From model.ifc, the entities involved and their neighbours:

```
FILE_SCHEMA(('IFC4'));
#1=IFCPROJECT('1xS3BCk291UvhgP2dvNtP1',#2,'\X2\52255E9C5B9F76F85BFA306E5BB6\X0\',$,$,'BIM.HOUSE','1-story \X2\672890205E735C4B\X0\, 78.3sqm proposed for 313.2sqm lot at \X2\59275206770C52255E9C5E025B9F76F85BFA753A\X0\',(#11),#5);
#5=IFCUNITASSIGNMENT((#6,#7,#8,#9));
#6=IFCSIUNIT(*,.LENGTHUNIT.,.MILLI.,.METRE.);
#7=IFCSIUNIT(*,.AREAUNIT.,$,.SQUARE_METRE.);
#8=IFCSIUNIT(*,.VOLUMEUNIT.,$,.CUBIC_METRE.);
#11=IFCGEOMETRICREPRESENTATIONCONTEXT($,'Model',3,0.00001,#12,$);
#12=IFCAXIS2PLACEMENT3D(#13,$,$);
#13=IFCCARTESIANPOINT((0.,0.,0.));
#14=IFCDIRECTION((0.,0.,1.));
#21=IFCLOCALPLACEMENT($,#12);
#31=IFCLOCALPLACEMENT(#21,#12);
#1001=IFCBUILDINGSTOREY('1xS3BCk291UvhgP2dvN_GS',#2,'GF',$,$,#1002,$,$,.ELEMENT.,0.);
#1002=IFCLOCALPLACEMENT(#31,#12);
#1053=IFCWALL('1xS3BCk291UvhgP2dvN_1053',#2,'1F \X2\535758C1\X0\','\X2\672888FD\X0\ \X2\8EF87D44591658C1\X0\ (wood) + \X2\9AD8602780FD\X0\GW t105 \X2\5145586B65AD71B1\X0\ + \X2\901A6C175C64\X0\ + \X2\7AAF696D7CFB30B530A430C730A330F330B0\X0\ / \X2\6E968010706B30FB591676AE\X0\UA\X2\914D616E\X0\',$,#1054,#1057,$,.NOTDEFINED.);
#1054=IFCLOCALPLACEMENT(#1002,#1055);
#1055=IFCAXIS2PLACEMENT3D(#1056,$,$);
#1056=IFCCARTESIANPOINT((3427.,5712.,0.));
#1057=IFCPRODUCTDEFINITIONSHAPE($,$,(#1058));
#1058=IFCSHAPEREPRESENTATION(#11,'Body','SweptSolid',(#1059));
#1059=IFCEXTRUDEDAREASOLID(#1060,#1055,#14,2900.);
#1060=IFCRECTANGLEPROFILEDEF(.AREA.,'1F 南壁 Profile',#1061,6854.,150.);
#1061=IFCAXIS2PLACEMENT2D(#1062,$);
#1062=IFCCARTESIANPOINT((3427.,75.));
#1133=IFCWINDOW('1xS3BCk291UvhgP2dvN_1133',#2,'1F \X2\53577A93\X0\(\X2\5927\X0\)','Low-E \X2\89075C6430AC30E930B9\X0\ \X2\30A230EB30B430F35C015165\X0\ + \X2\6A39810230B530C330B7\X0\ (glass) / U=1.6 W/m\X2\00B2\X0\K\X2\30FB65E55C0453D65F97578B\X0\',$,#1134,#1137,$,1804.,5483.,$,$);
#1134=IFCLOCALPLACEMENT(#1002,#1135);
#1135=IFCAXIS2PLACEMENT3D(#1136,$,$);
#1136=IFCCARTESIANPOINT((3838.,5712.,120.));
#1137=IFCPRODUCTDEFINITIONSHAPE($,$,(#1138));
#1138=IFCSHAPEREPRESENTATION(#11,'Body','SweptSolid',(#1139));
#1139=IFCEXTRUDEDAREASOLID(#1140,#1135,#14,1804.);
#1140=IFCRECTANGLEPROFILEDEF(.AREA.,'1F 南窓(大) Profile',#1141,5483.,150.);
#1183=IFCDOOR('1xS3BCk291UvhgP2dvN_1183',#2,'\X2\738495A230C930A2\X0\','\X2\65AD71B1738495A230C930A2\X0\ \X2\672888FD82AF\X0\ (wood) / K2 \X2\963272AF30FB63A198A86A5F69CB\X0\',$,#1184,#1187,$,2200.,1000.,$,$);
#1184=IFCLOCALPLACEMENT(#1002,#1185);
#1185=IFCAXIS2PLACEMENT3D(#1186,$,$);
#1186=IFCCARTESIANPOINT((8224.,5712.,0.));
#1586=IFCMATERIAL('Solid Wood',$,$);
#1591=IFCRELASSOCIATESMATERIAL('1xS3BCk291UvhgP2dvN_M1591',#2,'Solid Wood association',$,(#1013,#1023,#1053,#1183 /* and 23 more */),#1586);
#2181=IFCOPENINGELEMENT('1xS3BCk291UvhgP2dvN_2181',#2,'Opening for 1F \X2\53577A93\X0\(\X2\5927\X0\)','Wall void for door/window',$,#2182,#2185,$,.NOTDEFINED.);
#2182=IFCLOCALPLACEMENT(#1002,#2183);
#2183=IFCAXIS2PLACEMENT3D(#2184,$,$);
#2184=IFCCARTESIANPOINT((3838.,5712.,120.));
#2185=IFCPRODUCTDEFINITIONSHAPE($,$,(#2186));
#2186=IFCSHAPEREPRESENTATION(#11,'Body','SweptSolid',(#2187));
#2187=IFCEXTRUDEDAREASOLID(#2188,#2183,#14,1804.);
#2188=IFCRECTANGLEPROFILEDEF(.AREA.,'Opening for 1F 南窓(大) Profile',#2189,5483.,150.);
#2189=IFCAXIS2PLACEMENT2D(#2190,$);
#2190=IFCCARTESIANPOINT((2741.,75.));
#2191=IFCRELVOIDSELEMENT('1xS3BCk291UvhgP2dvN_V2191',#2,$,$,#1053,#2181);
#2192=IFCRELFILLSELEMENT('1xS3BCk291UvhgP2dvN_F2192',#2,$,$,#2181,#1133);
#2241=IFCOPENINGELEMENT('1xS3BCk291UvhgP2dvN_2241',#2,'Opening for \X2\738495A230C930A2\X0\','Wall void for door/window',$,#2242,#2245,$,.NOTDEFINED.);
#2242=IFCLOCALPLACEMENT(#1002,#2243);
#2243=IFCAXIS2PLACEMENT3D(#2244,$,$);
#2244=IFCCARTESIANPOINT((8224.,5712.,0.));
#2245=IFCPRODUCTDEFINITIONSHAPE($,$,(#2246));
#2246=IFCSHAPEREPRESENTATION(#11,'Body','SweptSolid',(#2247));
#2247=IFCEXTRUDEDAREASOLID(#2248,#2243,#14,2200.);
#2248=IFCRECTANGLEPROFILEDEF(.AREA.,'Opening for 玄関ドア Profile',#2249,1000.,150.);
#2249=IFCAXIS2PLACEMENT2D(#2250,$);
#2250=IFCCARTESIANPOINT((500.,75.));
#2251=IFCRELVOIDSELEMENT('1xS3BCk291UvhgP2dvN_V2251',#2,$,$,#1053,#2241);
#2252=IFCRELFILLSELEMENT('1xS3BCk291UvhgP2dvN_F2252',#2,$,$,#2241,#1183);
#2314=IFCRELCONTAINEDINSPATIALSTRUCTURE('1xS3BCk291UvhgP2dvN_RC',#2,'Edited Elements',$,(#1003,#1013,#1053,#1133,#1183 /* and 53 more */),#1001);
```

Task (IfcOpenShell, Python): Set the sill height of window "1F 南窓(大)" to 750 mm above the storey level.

```python
import numpy as np
import ifcopenshell
import ifcopenshell.api.geometry
import ifcopenshell.geom
import ifcopenshell.util.element
import ifcopenshell.util.placement
import ifcopenshell.util.shape
import ifcopenshell.util.unit

model = ifcopenshell.open("model.ifc")
unit_scale = ifcopenshell.util.unit.calculate_unit_scale(model)

window = model.by_id(1133)
opening = window.FillsVoids[0].RelatingOpeningElement
storey = ifcopenshell.util.element.get_container(window, ifc_class="IfcBuildingStorey")
level = ifcopenshell.util.placement.get_local_placement(storey.ObjectPlacement)[2, 3]

# The opening's origin need not be at the sill, so measure its lowest point.
shape = ifcopenshell.geom.create_shape(ifcopenshell.geom.settings(), opening)
bottom = ifcopenshell.util.shape.get_shape_bottom_elevation(shape, shape.geometry) / unit_scale
dz = level + 0.75 / unit_scale - bottom

shift = np.array([0.0, 0.0, dz])
# The window is not placed relative to its opening, so move both.
for product in (opening, window):
    matrix = ifcopenshell.util.placement.get_local_placement(product.ObjectPlacement)
    matrix[:3, 3] += shift
    ifcopenshell.api.geometry.edit_object_placement(model, product=product, matrix=matrix, is_si=False)

print(f"moved by {dz * unit_scale:+.3f} m")

model.write("model_edited.ifc")
```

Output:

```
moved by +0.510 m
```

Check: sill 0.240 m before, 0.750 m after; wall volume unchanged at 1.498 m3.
